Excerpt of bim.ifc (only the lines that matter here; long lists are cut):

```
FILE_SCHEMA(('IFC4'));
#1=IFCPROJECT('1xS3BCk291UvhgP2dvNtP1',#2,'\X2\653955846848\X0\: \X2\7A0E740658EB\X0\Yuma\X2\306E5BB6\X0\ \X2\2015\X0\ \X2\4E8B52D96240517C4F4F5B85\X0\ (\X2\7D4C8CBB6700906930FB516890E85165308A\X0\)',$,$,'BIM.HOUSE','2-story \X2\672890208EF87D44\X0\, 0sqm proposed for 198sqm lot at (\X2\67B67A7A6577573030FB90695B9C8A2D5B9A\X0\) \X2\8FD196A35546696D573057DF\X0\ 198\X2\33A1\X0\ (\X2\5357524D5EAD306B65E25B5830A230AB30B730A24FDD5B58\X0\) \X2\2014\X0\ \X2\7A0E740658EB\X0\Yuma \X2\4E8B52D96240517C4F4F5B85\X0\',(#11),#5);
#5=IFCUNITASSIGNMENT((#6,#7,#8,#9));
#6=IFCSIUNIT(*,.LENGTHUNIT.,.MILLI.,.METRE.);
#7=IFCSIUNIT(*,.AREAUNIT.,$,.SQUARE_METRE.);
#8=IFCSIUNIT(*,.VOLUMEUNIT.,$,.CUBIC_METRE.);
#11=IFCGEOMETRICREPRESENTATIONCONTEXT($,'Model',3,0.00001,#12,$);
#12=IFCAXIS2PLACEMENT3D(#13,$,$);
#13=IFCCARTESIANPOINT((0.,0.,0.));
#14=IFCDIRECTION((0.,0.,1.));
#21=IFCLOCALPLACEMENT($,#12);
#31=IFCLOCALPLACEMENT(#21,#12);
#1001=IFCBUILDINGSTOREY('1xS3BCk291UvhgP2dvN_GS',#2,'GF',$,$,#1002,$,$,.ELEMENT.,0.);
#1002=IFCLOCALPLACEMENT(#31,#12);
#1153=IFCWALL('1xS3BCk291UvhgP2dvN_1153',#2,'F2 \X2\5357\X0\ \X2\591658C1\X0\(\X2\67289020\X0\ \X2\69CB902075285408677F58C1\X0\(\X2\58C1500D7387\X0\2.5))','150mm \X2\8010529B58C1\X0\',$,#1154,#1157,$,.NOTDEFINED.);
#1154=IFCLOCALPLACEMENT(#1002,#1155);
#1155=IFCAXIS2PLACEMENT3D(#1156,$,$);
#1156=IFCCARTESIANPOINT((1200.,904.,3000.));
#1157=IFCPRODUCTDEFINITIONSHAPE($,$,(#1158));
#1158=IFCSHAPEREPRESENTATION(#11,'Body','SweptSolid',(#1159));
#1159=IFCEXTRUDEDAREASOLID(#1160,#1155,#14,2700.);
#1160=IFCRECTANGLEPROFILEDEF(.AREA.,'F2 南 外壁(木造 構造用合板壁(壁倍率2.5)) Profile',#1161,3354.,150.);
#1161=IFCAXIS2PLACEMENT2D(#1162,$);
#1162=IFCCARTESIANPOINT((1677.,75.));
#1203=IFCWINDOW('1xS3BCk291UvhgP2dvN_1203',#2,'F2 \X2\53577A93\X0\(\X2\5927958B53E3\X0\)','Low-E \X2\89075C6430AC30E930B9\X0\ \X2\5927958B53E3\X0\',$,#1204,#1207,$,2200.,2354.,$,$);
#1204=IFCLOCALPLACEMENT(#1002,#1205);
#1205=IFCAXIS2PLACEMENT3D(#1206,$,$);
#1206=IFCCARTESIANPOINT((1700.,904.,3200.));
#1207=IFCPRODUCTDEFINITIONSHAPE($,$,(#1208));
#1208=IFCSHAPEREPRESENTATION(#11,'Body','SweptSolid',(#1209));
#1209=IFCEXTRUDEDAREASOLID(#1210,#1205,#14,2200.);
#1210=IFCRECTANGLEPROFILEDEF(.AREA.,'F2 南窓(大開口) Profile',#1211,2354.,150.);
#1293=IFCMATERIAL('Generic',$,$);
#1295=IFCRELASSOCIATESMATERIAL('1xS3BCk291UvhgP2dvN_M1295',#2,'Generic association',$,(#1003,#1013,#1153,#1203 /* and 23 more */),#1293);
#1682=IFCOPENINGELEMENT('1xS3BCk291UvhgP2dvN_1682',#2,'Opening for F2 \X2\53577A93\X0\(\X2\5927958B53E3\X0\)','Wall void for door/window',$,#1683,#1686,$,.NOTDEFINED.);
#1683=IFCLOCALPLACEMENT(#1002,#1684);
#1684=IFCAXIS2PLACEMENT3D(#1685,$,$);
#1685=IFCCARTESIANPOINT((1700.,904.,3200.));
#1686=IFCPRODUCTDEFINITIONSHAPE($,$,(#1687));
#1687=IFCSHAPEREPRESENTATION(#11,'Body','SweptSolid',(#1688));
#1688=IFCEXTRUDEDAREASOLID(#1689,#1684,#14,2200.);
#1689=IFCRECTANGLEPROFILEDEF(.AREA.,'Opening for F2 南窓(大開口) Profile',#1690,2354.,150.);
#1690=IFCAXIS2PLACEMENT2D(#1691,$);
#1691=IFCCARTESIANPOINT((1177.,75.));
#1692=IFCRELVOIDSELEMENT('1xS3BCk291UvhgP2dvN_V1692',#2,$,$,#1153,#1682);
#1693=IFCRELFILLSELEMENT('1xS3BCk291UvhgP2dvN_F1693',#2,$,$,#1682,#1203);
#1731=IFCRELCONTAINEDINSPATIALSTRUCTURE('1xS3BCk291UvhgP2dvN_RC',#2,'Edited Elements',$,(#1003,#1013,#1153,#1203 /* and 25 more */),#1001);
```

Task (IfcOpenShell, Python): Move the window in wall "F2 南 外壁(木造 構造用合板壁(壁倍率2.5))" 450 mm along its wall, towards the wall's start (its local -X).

```python
import ifcopenshell
import ifcopenshell.api.geometry
import ifcopenshell.util.placement
import ifcopenshell.util.unit

model = ifcopenshell.open("bim.ifc")
unit_scale = ifcopenshell.util.unit.calculate_unit_scale(model)

window = model.by_guid("1xS3BCk291UvhgP2dvN_1203")
opening = window.FillsVoids[0].RelatingOpeningElement
wall = opening.VoidsElements[0].RelatingBuildingElement

wall_matrix = ifcopenshell.util.placement.get_local_placement(wall.ObjectPlacement)
shift = wall_matrix[:3, 0] * -0.45 / unit_scale
before = ifcopenshell.util.placement.get_local_placement(window.ObjectPlacement)[:3, 3].copy()

# The window is not placed relative to its opening, so move both.
for product in (opening, window):
    matrix = ifcopenshell.util.placement.get_local_placement(product.ObjectPlacement)
    matrix[:3, 3] += shift
    ifcopenshell.api.geometry.edit_object_placement(model, product=product, matrix=matrix, is_si=False)

after = ifcopenshell.util.placement.get_local_placement(window.ObjectPlacement)[:3, 3]
print("window moved by", (after - before).round(3) + 0.0)

model.write("bim_v2.ifc")
```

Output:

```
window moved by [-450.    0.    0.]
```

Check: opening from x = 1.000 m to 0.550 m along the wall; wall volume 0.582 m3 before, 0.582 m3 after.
